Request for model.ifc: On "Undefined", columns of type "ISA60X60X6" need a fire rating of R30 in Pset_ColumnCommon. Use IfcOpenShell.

First a look at what the model holds.

```python
import ifcopenshell
import ifcopenshell.util.element

model = ifcopenshell.open("model.ifc")
print(model.schema)
storey = next(s for s in model.by_type("IfcBuildingStorey") if s.Name == "Undefined")
columns = [e for e in ifcopenshell.util.element.get_decomposition(storey) if e.is_a("IfcColumn")]
seen = {}
for e in columns:
    element_type = ifcopenshell.util.element.get_type(e)
    key = (element_type.Name if element_type != e and element_type else None, ifcopenshell.util.element.get_pset(e, "Pset_ColumnCommon", "FireRating"))
    seen[key] = seen.get(key, 0) + 1
for (name, value), count in sorted(seen.items(), key=str):
    print(count, "x", name, "|", value)
```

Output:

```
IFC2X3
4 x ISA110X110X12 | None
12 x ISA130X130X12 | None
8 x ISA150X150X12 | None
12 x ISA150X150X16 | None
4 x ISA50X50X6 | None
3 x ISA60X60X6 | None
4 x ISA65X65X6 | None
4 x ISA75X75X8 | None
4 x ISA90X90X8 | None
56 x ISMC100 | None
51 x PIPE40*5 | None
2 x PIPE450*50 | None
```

```python
import ifcopenshell
import ifcopenshell.api.pset
import ifcopenshell.util.element

model = ifcopenshell.open("model.ifc")

storey = next(s for s in model.by_type("IfcBuildingStorey") if s.Name == "Undefined")
columns = [e for e in ifcopenshell.util.element.get_decomposition(storey) if e.is_a("IfcColumn")]

count = 0
for e in columns:
    element_type = ifcopenshell.util.element.get_type(e)
    if element_type in (None, e) or element_type.Name != "ISA60X60X6":
        continue
    found = ifcopenshell.util.element.get_pset(e, "Pset_ColumnCommon", should_inherit=False)
    if found:
        pset = model.by_id(found["id"])
        if len(ifcopenshell.util.element.get_elements_by_pset(pset)) > 1:
            pset = ifcopenshell.api.pset.unshare_pset(model, products=[e], pset=pset)[0]
    else:
        pset = ifcopenshell.api.pset.add_pset(model, product=e, name="Pset_ColumnCommon")
    ifcopenshell.api.pset.edit_pset(model, pset=pset, properties={"FireRating": "R30"})
    count += 1

print(count, "columns updated")

model.write("model_edited.ifc")
```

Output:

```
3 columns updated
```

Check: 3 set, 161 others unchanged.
